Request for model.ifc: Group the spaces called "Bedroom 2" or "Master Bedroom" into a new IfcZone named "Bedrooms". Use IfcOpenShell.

First a look at what the model holds.

```python
import ifcopenshell

model = ifcopenshell.open("model.ifc")
print(model.schema)
seen = {}
for space in model.by_type("IfcSpace"):
    seen[space.LongName] = seen.get(space.LongName, 0) + 1
for name, count in sorted(seen.items(), key=str):
    print(count, "x", name)
print("zones:", [z.Name for z in model.by_type("IfcZone")][:20])
```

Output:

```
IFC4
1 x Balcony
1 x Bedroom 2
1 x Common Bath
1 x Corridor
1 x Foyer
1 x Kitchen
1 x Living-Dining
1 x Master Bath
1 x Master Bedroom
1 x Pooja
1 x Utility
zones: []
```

```python
import ifcopenshell
import ifcopenshell.api.group
import ifcopenshell.api.root

model = ifcopenshell.open("model.ifc")

names = {"Bedroom 2", "Master Bedroom"}
spaces = [s for s in model.by_type("IfcSpace") if s.LongName in names]

zone = ifcopenshell.api.root.create_entity(model, ifc_class="IfcZone", name="Bedrooms")
ifcopenshell.api.group.assign_group(model, products=spaces, group=zone)
print(len(spaces), "spaces in", zone.Name)

model.write("model_updated.ifc")
```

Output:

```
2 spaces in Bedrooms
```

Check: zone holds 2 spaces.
